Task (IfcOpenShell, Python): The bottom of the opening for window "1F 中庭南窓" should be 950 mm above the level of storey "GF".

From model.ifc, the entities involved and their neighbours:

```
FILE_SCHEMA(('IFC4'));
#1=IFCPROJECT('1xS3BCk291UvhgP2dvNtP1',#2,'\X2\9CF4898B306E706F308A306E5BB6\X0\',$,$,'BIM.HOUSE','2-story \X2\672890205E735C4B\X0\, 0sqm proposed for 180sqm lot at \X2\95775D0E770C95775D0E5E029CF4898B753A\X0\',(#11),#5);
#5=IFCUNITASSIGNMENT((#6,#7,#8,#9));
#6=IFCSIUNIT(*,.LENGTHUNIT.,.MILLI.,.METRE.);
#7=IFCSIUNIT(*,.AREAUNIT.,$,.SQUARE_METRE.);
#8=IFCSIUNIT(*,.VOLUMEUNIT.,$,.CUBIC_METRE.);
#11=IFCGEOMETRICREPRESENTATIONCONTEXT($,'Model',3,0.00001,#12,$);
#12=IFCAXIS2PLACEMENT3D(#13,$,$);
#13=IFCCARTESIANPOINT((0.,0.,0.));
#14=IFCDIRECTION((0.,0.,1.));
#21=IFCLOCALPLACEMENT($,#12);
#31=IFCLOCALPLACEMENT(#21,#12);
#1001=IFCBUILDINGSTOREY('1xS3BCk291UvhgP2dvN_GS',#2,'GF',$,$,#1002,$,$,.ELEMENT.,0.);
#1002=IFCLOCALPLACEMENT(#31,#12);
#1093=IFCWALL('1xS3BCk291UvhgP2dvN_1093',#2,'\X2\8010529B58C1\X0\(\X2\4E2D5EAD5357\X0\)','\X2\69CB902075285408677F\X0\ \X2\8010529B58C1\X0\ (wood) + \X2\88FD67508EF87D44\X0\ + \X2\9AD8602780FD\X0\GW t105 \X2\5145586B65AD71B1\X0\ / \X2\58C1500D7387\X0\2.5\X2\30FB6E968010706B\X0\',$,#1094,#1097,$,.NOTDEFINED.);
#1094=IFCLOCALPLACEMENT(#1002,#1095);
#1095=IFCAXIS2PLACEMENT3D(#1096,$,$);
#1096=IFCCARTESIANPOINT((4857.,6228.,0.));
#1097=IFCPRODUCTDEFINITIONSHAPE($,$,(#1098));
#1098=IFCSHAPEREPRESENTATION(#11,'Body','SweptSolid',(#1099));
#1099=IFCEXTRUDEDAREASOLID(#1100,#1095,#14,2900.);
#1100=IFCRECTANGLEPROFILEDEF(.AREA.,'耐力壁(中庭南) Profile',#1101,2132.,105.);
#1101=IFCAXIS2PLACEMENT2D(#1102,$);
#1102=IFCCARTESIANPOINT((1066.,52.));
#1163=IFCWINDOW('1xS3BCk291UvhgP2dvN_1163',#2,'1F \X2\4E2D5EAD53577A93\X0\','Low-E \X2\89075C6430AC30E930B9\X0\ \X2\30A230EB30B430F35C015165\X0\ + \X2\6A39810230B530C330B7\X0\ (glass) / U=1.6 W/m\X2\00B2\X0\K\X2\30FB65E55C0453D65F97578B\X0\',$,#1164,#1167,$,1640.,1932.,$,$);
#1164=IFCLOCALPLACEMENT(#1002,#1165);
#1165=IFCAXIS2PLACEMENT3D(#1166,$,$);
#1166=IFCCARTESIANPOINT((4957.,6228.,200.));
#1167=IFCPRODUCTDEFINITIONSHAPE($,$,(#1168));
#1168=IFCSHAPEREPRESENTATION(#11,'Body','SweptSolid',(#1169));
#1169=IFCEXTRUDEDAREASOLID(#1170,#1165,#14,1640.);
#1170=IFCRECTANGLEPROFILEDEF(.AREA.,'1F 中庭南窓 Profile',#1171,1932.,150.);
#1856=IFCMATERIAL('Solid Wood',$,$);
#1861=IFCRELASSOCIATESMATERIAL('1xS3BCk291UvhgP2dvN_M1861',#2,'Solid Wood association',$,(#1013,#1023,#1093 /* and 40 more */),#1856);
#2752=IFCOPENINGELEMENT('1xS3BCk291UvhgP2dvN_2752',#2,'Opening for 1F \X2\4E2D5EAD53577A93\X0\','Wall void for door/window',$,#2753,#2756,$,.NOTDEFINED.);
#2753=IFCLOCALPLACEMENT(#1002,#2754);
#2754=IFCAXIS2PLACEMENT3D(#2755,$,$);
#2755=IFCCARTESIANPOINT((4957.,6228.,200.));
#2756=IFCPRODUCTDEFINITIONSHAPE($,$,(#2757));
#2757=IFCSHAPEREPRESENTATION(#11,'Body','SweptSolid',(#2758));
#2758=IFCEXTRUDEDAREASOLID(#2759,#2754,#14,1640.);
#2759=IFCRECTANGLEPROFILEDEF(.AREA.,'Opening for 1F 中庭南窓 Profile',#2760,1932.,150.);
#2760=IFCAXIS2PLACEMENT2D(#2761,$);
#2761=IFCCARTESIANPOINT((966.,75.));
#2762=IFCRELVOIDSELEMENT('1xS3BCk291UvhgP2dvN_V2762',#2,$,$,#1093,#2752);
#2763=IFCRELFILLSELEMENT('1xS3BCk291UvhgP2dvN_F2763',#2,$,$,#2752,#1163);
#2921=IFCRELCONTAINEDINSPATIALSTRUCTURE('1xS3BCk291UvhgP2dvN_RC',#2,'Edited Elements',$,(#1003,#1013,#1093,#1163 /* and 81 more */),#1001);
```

```python
import numpy as np
import ifcopenshell
import ifcopenshell.api.geometry
import ifcopenshell.geom
import ifcopenshell.util.element
import ifcopenshell.util.placement
import ifcopenshell.util.shape
import ifcopenshell.util.unit

model = ifcopenshell.open("model.ifc")
unit_scale = ifcopenshell.util.unit.calculate_unit_scale(model)

window = model.by_id(1163)
opening = window.FillsVoids[0].RelatingOpeningElement
storey = ifcopenshell.util.element.get_container(window, ifc_class="IfcBuildingStorey")
level = ifcopenshell.util.placement.get_local_placement(storey.ObjectPlacement)[2, 3]

# The opening's origin need not be at the sill, so measure its lowest point.
shape = ifcopenshell.geom.create_shape(ifcopenshell.geom.settings(), opening)
bottom = ifcopenshell.util.shape.get_shape_bottom_elevation(shape, shape.geometry) / unit_scale
dz = level + 0.95 / unit_scale - bottom

shift = np.array([0.0, 0.0, dz])
# The window is not placed relative to its opening, so move both.
for product in (opening, window):
    matrix = ifcopenshell.util.placement.get_local_placement(product.ObjectPlacement)
    matrix[:3, 3] += shift
    ifcopenshell.api.geometry.edit_object_placement(model, product=product, matrix=matrix, is_si=False)

print(f"moved by {dz * unit_scale:+.3f} m")

model.write("model-out.ifc")
```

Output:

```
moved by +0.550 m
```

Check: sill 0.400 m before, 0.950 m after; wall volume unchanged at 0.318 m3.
